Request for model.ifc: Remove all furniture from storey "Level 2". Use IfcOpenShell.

First a look at what the model holds.

```python
import ifcopenshell
import ifcopenshell.util.element

model = ifcopenshell.open("model.ifc")
print(model.schema)
storey = next(s for s in model.by_type("IfcBuildingStorey") if s.Name == "Level 2")
furniture = [e for e in ifcopenshell.util.element.get_decomposition(storey) if e.is_a("IfcFurnishingElement")]
seen = {}
for e in furniture:
    element_type = ifcopenshell.util.element.get_type(e)
    name = element_type.Name if element_type not in (None, e) else None
    seen[name] = seen.get(name, 0) + 1
for name, count in sorted(seen.items(), key=str):
    print(count, "x", name)
```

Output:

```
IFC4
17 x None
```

```python
import ifcopenshell
import ifcopenshell.api.root
import ifcopenshell.util.element

model = ifcopenshell.open("model.ifc")

storey = next(s for s in model.by_type("IfcBuildingStorey") if s.Name == "Level 2")
furniture = [e for e in ifcopenshell.util.element.get_decomposition(storey) if e.is_a("IfcFurnishingElement")]

for e in furniture:
    ifcopenshell.api.root.remove_product(model, product=e)
print(len(furniture), "removed")

model.write("model_updated.ifc")
```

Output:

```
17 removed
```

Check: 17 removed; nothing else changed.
